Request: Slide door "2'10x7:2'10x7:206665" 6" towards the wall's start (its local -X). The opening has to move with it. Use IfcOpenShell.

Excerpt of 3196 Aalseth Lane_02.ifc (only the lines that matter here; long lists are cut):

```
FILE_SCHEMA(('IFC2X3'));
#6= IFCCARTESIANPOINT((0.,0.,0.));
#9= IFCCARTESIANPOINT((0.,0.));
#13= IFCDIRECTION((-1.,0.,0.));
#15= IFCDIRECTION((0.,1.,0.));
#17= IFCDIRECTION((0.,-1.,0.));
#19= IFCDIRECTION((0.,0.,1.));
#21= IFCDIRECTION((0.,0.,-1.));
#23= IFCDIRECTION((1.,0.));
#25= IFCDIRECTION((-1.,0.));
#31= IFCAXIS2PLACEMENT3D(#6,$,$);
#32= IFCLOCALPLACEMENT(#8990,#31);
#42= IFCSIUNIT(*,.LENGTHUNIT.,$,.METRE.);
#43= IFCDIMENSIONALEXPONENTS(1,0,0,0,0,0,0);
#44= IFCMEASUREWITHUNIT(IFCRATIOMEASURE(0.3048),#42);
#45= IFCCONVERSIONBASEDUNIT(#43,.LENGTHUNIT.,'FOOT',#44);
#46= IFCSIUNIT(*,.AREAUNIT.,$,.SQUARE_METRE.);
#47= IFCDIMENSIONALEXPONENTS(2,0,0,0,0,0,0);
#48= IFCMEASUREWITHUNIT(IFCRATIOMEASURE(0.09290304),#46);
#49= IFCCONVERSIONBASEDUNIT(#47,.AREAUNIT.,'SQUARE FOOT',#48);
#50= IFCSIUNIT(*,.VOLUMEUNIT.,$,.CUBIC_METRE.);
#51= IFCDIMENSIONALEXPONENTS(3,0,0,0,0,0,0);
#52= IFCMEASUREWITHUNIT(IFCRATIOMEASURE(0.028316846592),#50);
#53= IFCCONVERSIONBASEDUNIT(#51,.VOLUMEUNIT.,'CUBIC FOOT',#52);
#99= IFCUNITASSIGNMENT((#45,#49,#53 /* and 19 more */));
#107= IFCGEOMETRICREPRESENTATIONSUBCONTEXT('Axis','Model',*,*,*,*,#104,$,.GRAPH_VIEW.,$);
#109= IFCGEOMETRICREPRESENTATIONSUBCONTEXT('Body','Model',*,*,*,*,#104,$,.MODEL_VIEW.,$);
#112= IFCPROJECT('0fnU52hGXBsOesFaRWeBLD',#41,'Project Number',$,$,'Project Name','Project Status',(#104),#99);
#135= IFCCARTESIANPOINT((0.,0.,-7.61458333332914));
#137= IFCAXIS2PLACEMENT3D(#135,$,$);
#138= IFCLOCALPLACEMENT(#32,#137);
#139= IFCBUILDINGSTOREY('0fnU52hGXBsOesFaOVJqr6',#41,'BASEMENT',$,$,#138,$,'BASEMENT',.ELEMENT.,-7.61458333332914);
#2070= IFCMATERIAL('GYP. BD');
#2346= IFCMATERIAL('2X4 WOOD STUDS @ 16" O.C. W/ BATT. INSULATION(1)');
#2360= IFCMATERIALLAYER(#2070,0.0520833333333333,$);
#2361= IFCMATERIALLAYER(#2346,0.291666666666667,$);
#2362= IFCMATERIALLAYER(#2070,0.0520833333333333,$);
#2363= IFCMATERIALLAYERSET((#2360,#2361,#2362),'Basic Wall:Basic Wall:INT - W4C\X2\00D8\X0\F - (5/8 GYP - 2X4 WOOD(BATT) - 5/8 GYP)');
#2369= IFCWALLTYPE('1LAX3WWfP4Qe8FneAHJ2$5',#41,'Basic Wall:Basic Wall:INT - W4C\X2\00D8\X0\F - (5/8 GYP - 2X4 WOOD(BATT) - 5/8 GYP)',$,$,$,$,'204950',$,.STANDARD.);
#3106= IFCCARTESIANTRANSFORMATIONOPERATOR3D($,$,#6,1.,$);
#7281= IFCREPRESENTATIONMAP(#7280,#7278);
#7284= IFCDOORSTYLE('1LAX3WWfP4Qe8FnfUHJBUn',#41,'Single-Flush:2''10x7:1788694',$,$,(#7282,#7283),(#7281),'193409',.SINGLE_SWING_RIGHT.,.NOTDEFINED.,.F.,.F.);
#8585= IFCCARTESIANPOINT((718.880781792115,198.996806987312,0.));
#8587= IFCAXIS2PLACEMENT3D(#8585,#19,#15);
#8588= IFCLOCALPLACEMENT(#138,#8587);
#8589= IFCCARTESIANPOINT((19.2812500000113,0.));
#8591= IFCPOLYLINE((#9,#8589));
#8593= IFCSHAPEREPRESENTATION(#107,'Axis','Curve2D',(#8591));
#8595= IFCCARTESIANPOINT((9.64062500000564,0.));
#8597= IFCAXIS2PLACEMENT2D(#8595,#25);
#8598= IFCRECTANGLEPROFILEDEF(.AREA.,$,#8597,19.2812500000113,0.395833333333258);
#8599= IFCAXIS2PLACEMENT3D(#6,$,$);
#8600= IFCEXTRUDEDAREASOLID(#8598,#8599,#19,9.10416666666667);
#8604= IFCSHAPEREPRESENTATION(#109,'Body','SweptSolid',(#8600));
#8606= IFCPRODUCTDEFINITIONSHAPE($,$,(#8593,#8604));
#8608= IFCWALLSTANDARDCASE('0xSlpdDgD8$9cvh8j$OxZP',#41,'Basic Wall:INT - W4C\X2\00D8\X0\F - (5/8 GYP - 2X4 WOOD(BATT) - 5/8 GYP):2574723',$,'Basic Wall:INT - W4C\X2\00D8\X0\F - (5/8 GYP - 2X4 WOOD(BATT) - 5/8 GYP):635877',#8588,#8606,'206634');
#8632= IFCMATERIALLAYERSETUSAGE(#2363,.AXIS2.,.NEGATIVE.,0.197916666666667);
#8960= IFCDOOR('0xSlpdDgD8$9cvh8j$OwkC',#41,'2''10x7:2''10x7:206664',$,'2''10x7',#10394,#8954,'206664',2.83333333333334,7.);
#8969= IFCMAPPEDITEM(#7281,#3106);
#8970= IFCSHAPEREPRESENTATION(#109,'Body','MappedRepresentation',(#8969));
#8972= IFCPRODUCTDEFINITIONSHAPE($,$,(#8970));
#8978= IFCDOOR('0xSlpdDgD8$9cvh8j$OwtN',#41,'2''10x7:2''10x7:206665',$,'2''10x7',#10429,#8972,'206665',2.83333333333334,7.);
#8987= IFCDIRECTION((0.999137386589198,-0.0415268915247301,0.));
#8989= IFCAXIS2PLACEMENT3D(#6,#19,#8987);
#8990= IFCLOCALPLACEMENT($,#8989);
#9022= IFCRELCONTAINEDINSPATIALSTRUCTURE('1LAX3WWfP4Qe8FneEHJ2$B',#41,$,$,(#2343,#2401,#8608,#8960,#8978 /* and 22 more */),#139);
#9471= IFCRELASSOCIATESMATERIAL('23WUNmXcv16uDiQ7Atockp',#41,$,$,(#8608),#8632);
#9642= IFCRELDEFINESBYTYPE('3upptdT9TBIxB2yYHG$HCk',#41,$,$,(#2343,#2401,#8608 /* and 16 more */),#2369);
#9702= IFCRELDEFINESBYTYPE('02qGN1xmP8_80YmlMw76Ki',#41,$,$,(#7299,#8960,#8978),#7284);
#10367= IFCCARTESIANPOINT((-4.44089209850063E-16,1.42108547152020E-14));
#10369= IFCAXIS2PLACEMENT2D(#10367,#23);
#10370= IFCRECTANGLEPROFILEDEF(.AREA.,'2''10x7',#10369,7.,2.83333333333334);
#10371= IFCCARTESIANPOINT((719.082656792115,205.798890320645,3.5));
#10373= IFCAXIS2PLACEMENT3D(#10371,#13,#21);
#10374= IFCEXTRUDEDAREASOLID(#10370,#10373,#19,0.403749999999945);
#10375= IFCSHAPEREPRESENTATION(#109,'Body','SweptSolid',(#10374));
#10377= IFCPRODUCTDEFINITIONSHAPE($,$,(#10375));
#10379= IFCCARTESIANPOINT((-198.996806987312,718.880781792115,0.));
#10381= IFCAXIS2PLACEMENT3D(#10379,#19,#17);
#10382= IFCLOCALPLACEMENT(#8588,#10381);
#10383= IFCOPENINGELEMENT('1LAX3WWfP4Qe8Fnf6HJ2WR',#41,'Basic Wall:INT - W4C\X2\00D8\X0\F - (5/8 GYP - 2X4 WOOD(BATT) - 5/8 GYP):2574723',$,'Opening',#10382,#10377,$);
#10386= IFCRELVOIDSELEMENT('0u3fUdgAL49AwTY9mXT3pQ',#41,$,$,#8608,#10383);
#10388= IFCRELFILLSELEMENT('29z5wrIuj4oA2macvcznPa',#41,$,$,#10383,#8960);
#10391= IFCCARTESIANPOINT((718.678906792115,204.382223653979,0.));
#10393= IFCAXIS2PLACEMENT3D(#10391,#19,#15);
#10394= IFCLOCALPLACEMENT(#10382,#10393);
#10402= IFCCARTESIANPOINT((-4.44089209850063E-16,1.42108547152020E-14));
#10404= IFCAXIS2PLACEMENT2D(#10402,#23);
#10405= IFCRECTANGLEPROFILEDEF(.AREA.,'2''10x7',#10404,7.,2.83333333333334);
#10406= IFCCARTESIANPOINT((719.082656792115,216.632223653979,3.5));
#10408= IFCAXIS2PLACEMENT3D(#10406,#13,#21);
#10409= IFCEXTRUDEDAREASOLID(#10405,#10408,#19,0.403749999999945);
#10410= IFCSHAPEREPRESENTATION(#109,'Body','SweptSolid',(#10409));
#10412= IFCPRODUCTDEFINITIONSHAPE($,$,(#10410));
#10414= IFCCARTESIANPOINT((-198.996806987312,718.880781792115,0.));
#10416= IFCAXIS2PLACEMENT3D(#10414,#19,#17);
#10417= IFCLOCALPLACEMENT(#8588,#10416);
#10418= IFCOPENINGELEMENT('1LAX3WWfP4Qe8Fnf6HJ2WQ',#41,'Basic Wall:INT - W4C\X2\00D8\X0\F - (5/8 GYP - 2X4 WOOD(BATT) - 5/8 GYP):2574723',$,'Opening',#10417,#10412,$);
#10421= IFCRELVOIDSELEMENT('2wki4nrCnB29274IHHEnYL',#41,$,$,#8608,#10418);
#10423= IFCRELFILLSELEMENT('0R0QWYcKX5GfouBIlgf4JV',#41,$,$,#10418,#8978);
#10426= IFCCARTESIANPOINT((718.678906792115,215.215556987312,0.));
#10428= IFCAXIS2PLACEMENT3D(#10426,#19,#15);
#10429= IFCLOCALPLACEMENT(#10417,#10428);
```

```python
import ifcopenshell
import ifcopenshell.api.geometry
import ifcopenshell.util.placement
import ifcopenshell.util.unit

model = ifcopenshell.open("3196 Aalseth Lane_02.ifc")
unit_scale = ifcopenshell.util.unit.calculate_unit_scale(model)

door = model.by_guid("0xSlpdDgD8$9cvh8j$OwtN")
opening = door.FillsVoids[0].RelatingOpeningElement
wall = opening.VoidsElements[0].RelatingBuildingElement

wall_matrix = ifcopenshell.util.placement.get_local_placement(wall.ObjectPlacement)
shift = wall_matrix[:3, 0] * -6 * 0.0254 / unit_scale
before = ifcopenshell.util.placement.get_local_placement(door.ObjectPlacement)[:3, 3].copy()

# The door is placed relative to its opening, so it follows when the opening moves.
matrix = ifcopenshell.util.placement.get_local_placement(opening.ObjectPlacement)
matrix[:3, 3] += shift
ifcopenshell.api.geometry.edit_object_placement(
    model, product=opening, matrix=matrix, is_si=False, should_transform_children=True
)

after = ifcopenshell.util.placement.get_local_placement(door.ObjectPlacement)[:3, 3]
print("door moved by", (after - before).round(3) + 0.0)

model.write("3196 Aalseth Lane_02_updated.ifc")
```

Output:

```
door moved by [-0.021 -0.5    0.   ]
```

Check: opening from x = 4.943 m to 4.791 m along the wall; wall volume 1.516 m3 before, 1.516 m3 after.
